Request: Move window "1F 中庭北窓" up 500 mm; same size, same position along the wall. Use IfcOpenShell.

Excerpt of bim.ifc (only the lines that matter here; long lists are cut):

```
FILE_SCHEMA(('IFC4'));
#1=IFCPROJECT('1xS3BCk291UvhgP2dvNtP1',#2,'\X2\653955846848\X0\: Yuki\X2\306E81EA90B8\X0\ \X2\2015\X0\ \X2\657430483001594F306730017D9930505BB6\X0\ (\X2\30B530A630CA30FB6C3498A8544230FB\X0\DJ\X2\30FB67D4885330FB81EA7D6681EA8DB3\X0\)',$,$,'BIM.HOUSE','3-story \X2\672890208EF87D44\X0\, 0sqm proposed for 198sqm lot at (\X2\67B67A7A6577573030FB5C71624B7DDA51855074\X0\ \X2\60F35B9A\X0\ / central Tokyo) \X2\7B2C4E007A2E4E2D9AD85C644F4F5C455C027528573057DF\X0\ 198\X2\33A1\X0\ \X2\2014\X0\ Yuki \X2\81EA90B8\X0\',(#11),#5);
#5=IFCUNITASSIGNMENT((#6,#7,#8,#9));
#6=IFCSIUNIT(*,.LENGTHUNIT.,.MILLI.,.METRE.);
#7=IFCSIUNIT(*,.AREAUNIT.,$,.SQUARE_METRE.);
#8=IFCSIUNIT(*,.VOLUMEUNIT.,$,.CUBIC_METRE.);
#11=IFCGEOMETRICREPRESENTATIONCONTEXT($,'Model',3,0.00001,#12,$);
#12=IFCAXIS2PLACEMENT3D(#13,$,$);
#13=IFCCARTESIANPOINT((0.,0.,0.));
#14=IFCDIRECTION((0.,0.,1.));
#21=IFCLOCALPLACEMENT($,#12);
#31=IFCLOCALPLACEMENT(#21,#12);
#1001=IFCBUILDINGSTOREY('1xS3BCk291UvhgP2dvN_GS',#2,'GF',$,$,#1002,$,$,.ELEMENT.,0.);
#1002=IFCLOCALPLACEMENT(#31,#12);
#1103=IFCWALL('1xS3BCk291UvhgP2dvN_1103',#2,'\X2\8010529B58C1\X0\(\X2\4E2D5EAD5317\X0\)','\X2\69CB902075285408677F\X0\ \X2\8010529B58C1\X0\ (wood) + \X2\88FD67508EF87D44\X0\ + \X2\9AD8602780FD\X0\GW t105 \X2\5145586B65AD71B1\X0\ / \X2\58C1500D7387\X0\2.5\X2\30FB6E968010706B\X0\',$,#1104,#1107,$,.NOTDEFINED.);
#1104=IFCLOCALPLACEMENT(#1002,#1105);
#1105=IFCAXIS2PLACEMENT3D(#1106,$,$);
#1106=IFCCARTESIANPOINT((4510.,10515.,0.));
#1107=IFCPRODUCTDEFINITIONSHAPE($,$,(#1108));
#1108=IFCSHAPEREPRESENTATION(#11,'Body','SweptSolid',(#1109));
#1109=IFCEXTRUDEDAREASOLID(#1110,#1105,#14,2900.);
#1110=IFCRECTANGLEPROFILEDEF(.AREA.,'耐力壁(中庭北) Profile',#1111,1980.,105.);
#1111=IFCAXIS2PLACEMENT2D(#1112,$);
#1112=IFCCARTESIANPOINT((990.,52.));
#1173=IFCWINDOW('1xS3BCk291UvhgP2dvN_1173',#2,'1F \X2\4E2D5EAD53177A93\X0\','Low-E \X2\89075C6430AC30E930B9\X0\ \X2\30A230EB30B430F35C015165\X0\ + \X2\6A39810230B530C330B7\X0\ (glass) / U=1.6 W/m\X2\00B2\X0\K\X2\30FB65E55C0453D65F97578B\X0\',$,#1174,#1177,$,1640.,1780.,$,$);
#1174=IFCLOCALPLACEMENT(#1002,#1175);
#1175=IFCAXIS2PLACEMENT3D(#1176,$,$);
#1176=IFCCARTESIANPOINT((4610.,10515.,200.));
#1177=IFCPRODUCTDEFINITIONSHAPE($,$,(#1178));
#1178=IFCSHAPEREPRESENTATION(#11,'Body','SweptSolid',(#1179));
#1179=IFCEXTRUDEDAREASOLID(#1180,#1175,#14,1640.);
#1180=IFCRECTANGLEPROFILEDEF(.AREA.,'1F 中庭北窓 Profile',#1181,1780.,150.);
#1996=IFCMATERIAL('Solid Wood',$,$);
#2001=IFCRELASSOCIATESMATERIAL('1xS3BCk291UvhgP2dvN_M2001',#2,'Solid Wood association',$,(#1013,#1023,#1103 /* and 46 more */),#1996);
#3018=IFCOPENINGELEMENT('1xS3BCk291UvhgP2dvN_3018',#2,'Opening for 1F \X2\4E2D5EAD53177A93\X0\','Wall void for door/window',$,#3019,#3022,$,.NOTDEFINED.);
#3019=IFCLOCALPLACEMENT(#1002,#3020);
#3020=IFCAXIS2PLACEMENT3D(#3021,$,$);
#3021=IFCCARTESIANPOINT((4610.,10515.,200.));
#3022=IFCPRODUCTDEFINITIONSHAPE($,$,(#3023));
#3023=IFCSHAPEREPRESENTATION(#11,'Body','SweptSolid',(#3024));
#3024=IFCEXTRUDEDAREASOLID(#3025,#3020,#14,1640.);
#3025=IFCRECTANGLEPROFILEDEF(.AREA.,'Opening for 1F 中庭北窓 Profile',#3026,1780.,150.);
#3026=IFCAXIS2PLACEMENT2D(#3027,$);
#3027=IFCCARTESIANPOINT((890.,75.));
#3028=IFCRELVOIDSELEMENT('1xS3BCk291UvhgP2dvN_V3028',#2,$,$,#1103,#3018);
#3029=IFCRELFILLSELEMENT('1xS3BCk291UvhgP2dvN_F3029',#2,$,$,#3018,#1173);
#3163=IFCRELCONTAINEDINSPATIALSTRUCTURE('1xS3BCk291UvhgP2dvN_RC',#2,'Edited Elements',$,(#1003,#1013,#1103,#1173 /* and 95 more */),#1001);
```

```python
import numpy as np
import ifcopenshell
import ifcopenshell.api.geometry
import ifcopenshell.util.placement
import ifcopenshell.util.unit

model = ifcopenshell.open("bim.ifc")
unit_scale = ifcopenshell.util.unit.calculate_unit_scale(model)

window = model.by_guid("1xS3BCk291UvhgP2dvN_1173")
opening = window.FillsVoids[0].RelatingOpeningElement
dz = 0.5 / unit_scale

shift = np.array([0.0, 0.0, dz])
# The window is not placed relative to its opening, so move both.
for product in (opening, window):
    matrix = ifcopenshell.util.placement.get_local_placement(product.ObjectPlacement)
    matrix[:3, 3] += shift
    ifcopenshell.api.geometry.edit_object_placement(model, product=product, matrix=matrix, is_si=False)

print(f"moved by {dz * unit_scale:+.3f} m")

model.write("bim_updated.ifc")
```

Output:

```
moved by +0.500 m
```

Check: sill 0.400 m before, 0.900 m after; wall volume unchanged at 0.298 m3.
